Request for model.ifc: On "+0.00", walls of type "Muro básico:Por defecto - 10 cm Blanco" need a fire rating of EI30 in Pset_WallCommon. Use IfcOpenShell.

First a look at what the model holds.

```python
import ifcopenshell
import ifcopenshell.util.element

model = ifcopenshell.open("model.ifc")
print(model.schema)
storey = next(s for s in model.by_type("IfcBuildingStorey") if s.Name == "+0.00")
walls = [e for e in ifcopenshell.util.element.get_decomposition(storey) if e.is_a("IfcWall")]
seen = {}
for e in walls:
    element_type = ifcopenshell.util.element.get_type(e)
    key = (element_type.Name if element_type != e and element_type else None, ifcopenshell.util.element.get_pset(e, "Pset_WallCommon", "FireRating"))
    seen[key] = seen.get(key, 0) + 1
for (name, value), count in sorted(seen.items(), key=str):
    print(count, "x", name, "|", value)
```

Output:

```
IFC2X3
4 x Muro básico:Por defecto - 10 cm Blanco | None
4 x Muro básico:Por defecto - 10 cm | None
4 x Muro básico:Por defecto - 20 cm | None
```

```python
import ifcopenshell
import ifcopenshell.api.pset
import ifcopenshell.util.element

model = ifcopenshell.open("model.ifc")

storey = next(s for s in model.by_type("IfcBuildingStorey") if s.Name == "+0.00")
walls = [e for e in ifcopenshell.util.element.get_decomposition(storey) if e.is_a("IfcWall")]

count = 0
for e in walls:
    element_type = ifcopenshell.util.element.get_type(e)
    if element_type in (None, e) or element_type.Name != "Muro básico:Por defecto - 10 cm Blanco":
        continue
    # add_pset returns the element's existing set when there is one.
    pset = ifcopenshell.api.pset.add_pset(model, product=e, name="Pset_WallCommon")
    ifcopenshell.api.pset.edit_pset(model, pset=pset, properties={"FireRating": "EI30"})
    count += 1

print(count, "walls updated")

model.write("model-out.ifc")
```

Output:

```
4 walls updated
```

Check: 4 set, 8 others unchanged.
